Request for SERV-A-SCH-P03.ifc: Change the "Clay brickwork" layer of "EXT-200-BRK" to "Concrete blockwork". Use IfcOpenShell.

First a look at what the model holds.

```python
import ifcopenshell
import ifcopenshell.util.element

model = ifcopenshell.open("SERV-A-SCH-P03.ifc")
print(model.schema)
for layer_set in model.by_type("IfcMaterialLayerSet"):
    if layer_set.LayerSetName == "EXT-200-BRK":
        for layer in layer_set.MaterialLayers:
            print(layer.id(), layer.Material and layer.Material.Name, layer.LayerThickness, sep=" | ")
        print(len(ifcopenshell.util.element.get_elements_by_material(model, layer_set)), "elements and types use it")
print(sorted(m.Name for m in model.by_type("IfcMaterial") if m.Name)[:60])
```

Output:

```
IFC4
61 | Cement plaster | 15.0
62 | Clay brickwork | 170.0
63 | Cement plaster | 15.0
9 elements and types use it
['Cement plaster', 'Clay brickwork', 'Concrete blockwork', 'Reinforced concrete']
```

```python
import ifcopenshell
import ifcopenshell.api.material

model = ifcopenshell.open("SERV-A-SCH-P03.ifc")

layer_set = next(s for s in model.by_type("IfcMaterialLayerSet") if s.LayerSetName == "EXT-200-BRK")
layer = next(l for l in layer_set.MaterialLayers if l.Material and l.Material.Name == "Clay brickwork")
material = next(m for m in model.by_type("IfcMaterial") if m.Name == "Concrete blockwork")

# Point this one layer at the other material; renaming the old one would change it everywhere.
ifcopenshell.api.material.edit_layer(model, layer=layer, attributes={"Name": material.Name}, material=material)

print([l.Material.Name if l.Material else None for l in layer_set.MaterialLayers])

model.write("SERV-A-SCH-P03-out.ifc")
```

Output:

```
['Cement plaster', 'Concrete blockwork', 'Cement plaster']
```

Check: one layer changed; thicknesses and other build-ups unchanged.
